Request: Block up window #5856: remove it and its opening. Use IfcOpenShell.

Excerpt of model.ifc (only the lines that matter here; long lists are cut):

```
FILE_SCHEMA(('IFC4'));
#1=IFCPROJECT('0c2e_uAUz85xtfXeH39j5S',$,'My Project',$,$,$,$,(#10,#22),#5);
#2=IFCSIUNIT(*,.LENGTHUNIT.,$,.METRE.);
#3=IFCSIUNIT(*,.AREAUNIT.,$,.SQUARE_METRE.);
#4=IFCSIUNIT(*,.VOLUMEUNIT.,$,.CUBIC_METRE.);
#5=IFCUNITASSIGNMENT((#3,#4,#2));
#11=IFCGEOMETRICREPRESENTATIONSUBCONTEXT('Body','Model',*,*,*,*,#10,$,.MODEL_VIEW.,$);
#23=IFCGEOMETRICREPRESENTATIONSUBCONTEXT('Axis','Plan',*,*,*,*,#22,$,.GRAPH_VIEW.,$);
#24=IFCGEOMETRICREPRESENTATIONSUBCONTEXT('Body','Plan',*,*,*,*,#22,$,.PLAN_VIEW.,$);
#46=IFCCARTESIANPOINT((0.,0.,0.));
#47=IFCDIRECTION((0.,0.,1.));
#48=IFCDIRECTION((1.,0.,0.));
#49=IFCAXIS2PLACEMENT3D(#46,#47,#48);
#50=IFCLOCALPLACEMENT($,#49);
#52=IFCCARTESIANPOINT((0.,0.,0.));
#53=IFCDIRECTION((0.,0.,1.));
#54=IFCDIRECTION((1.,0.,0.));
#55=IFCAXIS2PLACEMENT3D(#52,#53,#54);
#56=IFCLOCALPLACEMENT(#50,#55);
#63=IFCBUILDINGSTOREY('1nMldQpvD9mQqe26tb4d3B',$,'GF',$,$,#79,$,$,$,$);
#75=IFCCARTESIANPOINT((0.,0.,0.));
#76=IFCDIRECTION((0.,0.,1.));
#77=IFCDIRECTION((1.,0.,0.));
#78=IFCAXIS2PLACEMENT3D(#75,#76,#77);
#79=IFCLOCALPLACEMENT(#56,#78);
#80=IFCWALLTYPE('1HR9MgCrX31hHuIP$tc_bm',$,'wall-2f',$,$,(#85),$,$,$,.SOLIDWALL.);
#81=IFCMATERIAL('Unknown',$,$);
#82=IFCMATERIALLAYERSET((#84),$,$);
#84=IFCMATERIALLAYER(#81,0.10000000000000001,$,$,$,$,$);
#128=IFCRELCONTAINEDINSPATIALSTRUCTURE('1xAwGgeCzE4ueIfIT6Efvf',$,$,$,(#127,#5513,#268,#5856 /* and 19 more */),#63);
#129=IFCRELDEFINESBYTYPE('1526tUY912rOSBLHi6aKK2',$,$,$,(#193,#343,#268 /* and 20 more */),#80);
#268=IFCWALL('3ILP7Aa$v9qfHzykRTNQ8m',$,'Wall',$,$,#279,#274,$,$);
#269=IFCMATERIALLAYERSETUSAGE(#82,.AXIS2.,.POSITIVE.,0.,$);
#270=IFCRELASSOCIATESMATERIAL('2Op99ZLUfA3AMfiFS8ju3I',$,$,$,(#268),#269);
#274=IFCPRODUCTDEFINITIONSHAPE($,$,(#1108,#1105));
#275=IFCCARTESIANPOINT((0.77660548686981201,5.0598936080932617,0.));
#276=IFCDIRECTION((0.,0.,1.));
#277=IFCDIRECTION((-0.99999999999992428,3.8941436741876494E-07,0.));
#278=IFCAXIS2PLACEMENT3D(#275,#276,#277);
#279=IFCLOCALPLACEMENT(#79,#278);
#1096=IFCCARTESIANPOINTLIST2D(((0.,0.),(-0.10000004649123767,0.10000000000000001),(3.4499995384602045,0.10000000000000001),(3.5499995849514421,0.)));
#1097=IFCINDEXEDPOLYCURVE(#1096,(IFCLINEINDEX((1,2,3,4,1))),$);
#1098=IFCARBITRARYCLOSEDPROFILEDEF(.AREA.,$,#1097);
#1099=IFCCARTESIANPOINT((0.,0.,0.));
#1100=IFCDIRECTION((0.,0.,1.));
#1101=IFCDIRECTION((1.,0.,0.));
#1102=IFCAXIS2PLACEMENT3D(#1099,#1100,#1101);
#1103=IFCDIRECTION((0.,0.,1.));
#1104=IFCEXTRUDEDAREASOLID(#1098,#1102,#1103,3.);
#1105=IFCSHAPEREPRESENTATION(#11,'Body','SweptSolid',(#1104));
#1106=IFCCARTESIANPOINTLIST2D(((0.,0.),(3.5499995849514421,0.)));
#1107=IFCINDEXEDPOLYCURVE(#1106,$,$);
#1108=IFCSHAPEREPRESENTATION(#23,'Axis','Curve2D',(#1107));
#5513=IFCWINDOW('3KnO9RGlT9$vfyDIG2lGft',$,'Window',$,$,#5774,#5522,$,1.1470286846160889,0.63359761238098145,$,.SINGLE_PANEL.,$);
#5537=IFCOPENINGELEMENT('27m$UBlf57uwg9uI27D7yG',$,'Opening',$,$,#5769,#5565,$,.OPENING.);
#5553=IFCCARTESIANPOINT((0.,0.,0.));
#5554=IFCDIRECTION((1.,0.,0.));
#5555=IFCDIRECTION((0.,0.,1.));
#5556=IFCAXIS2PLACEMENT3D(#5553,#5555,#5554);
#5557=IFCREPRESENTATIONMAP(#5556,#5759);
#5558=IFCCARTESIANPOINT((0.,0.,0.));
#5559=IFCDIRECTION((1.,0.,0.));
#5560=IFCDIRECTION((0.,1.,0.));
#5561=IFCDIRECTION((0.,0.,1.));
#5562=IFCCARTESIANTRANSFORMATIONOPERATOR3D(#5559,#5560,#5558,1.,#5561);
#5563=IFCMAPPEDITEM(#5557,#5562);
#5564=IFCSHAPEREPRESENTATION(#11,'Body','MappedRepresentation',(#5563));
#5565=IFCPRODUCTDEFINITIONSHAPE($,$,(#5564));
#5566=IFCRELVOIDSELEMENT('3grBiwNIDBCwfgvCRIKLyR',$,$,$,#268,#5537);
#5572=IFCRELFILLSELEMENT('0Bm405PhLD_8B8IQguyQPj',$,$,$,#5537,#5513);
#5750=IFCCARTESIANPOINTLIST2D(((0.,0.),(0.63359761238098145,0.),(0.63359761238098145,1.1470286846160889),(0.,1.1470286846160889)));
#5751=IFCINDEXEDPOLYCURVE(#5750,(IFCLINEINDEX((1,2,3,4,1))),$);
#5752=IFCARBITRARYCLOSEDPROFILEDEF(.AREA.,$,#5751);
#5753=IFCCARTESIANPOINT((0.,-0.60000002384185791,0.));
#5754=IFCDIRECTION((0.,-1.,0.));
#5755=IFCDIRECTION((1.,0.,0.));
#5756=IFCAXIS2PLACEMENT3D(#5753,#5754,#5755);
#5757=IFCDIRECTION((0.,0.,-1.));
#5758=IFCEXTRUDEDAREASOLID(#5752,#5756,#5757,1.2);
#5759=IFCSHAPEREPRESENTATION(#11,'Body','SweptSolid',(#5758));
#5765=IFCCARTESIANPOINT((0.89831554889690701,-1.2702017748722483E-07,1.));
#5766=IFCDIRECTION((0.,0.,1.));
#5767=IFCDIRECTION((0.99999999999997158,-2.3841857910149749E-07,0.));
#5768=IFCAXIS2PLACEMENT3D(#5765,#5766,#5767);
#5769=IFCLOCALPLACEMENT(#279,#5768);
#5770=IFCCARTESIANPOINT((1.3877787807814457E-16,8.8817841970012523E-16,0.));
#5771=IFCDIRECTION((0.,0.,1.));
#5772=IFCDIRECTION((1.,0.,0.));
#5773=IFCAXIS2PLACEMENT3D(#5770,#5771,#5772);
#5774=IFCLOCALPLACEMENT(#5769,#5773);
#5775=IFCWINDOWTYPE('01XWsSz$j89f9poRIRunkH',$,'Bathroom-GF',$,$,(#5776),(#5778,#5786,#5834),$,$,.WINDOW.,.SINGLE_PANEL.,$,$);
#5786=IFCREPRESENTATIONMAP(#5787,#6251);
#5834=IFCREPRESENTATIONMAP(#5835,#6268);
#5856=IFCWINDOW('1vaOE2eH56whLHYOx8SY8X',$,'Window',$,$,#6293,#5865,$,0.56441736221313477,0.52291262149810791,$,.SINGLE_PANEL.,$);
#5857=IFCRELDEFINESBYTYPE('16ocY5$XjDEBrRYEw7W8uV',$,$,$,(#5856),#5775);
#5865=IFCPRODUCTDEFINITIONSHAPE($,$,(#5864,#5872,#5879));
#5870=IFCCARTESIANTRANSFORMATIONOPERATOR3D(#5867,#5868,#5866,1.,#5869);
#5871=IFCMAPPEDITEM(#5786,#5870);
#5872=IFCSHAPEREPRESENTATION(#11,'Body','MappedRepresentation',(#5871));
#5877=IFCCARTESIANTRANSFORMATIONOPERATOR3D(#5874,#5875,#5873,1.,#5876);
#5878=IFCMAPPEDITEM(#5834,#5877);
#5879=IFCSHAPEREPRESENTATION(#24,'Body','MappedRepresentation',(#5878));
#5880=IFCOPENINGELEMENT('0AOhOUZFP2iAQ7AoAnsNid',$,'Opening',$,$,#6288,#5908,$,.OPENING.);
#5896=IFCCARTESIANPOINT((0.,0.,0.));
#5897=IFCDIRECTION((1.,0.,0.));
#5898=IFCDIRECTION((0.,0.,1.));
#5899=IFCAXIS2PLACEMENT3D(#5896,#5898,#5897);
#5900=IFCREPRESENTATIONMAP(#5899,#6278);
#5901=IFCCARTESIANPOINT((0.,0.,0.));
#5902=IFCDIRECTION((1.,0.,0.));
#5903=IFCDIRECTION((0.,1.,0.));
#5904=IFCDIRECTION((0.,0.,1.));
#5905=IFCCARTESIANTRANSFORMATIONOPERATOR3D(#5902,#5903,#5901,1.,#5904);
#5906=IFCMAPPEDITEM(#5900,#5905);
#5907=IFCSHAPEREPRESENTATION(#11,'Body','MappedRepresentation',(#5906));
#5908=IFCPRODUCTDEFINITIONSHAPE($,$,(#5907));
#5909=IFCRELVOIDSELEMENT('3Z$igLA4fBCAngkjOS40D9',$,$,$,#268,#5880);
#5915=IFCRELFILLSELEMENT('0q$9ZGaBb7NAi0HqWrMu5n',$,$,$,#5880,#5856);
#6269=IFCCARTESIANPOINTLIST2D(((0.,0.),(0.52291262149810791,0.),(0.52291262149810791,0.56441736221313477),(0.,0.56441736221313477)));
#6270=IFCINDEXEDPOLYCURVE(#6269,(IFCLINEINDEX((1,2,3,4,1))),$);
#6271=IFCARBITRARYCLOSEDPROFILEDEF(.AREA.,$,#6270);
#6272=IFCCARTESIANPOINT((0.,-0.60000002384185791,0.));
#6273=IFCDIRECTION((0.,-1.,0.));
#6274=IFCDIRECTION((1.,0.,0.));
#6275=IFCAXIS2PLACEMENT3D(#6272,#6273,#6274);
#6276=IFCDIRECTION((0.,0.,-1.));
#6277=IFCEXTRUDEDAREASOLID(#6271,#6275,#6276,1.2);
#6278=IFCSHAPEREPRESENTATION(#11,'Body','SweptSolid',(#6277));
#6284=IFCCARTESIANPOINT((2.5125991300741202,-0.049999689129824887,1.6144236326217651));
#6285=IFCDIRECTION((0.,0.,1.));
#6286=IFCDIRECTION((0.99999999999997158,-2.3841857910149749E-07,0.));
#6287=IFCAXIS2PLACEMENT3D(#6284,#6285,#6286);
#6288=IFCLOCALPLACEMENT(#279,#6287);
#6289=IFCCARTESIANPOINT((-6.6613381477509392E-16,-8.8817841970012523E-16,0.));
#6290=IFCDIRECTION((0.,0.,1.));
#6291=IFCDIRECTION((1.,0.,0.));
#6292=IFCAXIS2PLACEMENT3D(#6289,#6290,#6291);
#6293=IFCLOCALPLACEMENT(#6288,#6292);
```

```python
import ifcopenshell
import ifcopenshell.api.feature
import ifcopenshell.api.root
import ifcopenshell.geom
import ifcopenshell.util.shape

model = ifcopenshell.open("model.ifc")
settings = ifcopenshell.geom.settings()


def volume(element):
    """Net volume in cubic metres, openings subtracted."""
    shape = ifcopenshell.geom.create_shape(settings, element)
    return ifcopenshell.util.shape.get_volume(shape.geometry)


window = model.by_guid("1vaOE2eH56whLHYOx8SY8X")
opening = window.FillsVoids[0].RelatingOpeningElement
wall = opening.VoidsElements[0].RelatingBuildingElement
before = volume(wall)

ifcopenshell.api.root.remove_product(model, product=window)
ifcopenshell.api.feature.remove_feature(model, feature=opening)

after = volume(wall)

print(f"wall volume {before:.3f} -> {after:.3f} m3")

model.write("model_v2.ifc")
```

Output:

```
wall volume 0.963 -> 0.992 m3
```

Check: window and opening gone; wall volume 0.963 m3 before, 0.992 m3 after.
